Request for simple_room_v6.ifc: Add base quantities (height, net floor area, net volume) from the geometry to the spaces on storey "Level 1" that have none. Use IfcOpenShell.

First a look at what the model holds.

```python
import ifcopenshell
import ifcopenshell.util.element
import ifcopenshell.util.unit

model = ifcopenshell.open("simple_room_v6.ifc")
print(model.schema)
for unit_type in ("LENGTHUNIT", "AREAUNIT", "VOLUMEUNIT"):
    print(unit_type, ifcopenshell.util.unit.calculate_unit_scale(model, unit_type))
storey = next(s for s in model.by_type("IfcBuildingStorey") if s.Name == "Level 1")
spaces = [e for e in ifcopenshell.util.element.get_decomposition(storey) if e.is_a("IfcSpace")]
for e in sorted(spaces, key=lambda e: e.id()):
    print(e.id(), e.is_a(), e.Name, list(ifcopenshell.util.element.get_psets(e, qtos_only=True)), sep=" | ")
```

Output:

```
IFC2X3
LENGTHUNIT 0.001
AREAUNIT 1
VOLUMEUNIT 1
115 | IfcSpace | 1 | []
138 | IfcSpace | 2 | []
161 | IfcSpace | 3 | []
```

```python
import ifcopenshell
import ifcopenshell.api.pset
import ifcopenshell.geom
import ifcopenshell.util.element
import ifcopenshell.util.shape
import ifcopenshell.util.unit

model = ifcopenshell.open("simple_room_v6.ifc")
unit_scale = ifcopenshell.util.unit.calculate_unit_scale(model)
area_scale = ifcopenshell.util.unit.calculate_unit_scale(model, "AREAUNIT")
volume_scale = ifcopenshell.util.unit.calculate_unit_scale(model, "VOLUMEUNIT")
settings = ifcopenshell.geom.settings()

storey = next(s for s in model.by_type("IfcBuildingStorey") if s.Name == "Level 1")
spaces = [e for e in ifcopenshell.util.element.get_decomposition(storey) if e.is_a("IfcSpace")]

for e in sorted(spaces, key=lambda e: e.id()):
    if ifcopenshell.util.element.get_psets(e, qtos_only=True, should_inherit=False):
        continue
    # Geometry comes back in metres, in the element's own axes.
    shape = ifcopenshell.geom.create_shape(settings, e)
    values = {
        "Height": ifcopenshell.util.shape.get_z(shape.geometry) / unit_scale,
        "NetFloorArea": ifcopenshell.util.shape.get_footprint_area(shape.geometry) / area_scale,
        "NetVolume": ifcopenshell.util.shape.get_volume(shape.geometry) / volume_scale,
    }
    qto = ifcopenshell.api.pset.add_qto(model, product=e, name="BaseQuantities")
    ifcopenshell.api.pset.edit_qto(model, qto=qto, properties=values)
    print(e.id(), {k: round(v, 3) for k, v in values.items()})

model.write("simple_room_v6_edited.ifc")
```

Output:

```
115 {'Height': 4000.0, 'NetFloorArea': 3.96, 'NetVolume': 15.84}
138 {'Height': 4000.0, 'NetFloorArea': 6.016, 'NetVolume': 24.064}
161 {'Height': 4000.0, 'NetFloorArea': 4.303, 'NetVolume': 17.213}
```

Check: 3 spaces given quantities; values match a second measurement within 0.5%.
